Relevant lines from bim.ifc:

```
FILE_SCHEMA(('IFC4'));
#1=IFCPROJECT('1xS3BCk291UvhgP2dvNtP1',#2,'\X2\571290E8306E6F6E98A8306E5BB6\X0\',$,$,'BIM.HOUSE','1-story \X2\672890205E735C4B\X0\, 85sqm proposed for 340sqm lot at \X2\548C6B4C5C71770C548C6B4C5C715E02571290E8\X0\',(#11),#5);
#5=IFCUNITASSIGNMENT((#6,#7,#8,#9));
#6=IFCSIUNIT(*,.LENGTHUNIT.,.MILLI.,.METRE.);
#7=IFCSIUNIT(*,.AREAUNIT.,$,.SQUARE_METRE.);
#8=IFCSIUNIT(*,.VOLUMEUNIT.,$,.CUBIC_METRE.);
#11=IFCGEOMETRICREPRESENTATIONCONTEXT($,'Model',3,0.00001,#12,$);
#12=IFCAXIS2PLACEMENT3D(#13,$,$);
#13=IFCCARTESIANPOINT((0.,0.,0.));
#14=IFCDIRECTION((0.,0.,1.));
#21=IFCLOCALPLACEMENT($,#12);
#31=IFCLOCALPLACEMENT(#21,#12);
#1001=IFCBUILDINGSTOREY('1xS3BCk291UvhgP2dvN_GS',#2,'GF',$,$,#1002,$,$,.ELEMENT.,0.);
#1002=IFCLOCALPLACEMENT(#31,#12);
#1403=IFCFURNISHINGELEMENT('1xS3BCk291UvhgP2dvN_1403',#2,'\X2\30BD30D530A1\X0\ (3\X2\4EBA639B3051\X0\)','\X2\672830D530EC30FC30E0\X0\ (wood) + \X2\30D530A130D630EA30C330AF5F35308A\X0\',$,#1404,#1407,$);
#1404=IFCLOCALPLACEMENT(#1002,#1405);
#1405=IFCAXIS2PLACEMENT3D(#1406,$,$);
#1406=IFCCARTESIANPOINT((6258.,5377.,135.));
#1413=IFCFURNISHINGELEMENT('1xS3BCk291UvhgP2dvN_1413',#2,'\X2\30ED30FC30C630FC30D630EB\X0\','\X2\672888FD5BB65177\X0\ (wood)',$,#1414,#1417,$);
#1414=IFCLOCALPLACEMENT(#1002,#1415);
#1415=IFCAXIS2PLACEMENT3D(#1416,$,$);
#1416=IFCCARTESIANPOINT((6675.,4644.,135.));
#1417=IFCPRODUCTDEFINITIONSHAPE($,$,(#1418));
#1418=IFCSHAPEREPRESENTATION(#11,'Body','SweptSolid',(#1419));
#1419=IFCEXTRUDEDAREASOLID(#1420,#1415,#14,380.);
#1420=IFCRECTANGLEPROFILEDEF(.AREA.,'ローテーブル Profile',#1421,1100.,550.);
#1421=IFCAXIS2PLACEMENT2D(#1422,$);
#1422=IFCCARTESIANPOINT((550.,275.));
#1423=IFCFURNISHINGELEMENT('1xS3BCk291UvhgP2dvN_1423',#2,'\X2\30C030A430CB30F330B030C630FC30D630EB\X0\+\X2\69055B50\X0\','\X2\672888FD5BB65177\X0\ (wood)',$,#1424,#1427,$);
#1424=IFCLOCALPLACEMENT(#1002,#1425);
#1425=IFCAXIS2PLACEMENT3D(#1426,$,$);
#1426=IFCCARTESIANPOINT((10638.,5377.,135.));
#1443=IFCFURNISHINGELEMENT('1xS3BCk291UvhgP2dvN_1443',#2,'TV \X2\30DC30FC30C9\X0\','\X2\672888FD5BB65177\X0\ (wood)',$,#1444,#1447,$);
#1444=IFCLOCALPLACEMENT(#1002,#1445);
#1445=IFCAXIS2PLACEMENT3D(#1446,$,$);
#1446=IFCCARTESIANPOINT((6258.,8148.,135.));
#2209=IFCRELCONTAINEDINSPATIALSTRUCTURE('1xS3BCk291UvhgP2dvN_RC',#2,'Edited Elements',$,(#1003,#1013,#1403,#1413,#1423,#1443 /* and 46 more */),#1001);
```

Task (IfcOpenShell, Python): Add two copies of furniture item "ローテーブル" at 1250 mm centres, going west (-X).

```python
import numpy as np
import ifcopenshell
import ifcopenshell.api.geometry
import ifcopenshell.api.root
import ifcopenshell.util.element
import ifcopenshell.util.placement

model = ifcopenshell.open("bim.ifc")


def reuse_history(source, copy):
    """copy_class also copies each property set's owner history, people and application; keep the originals."""
    for rel in copy.IsDefinedBy:
        if rel.is_a("IfcRelDefinesByProperties") and (history := rel.RelatingPropertyDefinition.OwnerHistory):
            rel.RelatingPropertyDefinition.OwnerHistory = source.OwnerHistory
            ifcopenshell.util.element.remove_deep2(model, history)


source = model.by_guid("1xS3BCk291UvhgP2dvN_1413")
base = ifcopenshell.util.placement.get_local_placement(source.ObjectPlacement)
step = np.array([-1.0, 0.0, 0.0]) * 1250.0

for i in range(1, 3):
    copy = ifcopenshell.api.root.copy_class(model, product=source)
    copy.Representation = ifcopenshell.util.element.copy_deep(
        model, source.Representation, exclude=["IfcGeometricRepresentationContext", "IfcRepresentationMap"]
    )
    reuse_history(source, copy)
    matrix = base.copy()
    matrix[:3, 3] += i * step
    print("added at", matrix[:3, 3].round(3) + 0.0)
    ifcopenshell.api.geometry.edit_object_placement(model, product=copy, matrix=matrix, is_si=False)

model.write("bim_v2.ifc")
```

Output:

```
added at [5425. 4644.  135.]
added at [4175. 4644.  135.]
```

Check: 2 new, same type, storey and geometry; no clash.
